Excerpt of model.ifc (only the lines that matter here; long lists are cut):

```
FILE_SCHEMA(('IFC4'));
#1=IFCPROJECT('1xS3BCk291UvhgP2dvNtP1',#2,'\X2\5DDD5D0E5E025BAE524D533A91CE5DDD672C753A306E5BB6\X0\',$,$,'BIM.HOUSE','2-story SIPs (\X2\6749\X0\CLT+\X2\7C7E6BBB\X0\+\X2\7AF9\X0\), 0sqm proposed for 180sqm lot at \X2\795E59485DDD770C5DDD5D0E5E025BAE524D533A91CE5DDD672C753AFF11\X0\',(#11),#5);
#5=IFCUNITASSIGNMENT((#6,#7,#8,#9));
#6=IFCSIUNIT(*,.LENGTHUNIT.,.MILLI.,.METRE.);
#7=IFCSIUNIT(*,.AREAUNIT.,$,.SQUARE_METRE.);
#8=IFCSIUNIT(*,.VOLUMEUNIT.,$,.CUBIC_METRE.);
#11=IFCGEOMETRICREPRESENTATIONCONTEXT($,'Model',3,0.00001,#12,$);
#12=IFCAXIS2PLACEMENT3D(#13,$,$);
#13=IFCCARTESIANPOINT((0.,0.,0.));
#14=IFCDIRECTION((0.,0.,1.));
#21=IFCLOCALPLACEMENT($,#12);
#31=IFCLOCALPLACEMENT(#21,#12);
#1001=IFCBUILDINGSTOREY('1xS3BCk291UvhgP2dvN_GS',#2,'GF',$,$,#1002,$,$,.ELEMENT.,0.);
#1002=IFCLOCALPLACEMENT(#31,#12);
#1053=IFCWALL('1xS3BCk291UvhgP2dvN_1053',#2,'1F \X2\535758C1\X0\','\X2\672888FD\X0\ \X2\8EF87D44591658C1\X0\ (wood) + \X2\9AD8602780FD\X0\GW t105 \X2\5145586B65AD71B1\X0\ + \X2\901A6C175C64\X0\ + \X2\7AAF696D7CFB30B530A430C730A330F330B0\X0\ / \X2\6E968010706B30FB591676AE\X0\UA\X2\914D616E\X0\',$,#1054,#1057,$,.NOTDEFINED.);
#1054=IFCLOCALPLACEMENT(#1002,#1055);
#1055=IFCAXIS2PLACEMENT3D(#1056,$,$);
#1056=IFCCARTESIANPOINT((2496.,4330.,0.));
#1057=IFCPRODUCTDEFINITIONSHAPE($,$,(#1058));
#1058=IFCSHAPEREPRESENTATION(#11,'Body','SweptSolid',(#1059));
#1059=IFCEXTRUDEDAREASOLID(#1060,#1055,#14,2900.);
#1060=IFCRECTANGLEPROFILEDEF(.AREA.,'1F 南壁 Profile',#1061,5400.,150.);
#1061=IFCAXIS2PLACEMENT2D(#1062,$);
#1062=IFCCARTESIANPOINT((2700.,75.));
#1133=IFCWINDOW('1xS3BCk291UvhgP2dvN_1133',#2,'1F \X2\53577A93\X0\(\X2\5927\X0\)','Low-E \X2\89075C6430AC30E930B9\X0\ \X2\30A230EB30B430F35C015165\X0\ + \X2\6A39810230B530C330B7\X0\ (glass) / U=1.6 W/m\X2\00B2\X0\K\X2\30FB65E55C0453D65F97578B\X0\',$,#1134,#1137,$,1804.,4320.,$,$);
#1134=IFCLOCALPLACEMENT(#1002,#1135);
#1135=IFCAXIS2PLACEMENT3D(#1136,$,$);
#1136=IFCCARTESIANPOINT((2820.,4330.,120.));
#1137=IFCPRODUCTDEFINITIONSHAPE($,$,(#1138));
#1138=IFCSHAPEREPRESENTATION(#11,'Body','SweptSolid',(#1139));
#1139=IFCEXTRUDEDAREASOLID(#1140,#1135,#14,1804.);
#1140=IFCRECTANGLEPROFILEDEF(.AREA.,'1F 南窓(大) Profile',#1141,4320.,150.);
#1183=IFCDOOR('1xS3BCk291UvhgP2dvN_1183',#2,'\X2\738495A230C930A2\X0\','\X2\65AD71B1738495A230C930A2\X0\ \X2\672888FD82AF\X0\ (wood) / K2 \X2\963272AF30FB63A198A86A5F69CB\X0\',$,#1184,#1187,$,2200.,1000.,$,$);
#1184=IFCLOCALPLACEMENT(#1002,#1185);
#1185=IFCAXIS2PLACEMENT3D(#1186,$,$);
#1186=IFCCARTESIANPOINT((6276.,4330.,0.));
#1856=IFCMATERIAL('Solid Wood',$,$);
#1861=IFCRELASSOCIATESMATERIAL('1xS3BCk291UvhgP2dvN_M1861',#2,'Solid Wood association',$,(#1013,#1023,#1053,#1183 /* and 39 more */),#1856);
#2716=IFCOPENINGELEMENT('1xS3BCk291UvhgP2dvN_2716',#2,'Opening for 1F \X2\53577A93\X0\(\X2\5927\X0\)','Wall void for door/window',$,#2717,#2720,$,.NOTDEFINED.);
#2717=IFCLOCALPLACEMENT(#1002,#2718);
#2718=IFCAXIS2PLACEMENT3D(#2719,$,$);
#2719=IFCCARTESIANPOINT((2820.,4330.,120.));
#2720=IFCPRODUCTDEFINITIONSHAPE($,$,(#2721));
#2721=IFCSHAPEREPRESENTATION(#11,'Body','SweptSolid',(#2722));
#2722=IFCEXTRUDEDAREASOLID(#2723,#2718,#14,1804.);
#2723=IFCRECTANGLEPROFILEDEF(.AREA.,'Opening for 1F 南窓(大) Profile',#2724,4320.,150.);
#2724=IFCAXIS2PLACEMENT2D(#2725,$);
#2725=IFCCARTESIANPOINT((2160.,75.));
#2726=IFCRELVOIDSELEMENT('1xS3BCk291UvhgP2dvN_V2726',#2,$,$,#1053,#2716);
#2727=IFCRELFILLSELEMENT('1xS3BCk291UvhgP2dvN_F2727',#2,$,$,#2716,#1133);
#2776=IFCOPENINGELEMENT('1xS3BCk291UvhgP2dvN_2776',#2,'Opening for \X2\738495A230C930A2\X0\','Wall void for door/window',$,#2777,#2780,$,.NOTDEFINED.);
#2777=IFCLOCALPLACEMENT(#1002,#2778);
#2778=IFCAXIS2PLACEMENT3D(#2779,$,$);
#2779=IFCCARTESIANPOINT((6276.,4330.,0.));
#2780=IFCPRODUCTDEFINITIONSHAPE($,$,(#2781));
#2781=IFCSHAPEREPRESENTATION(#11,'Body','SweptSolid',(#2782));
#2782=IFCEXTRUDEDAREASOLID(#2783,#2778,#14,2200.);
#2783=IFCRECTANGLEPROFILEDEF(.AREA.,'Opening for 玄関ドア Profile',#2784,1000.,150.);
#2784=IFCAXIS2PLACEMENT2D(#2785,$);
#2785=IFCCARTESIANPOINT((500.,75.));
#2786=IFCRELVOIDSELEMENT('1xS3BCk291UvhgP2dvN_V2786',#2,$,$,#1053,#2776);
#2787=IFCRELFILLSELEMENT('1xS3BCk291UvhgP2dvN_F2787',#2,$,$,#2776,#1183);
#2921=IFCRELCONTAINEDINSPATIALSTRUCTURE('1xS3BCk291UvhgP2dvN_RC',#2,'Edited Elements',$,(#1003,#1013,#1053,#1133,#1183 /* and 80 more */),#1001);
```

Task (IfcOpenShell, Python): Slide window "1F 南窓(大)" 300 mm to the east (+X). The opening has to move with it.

```python
import ifcopenshell
import ifcopenshell.api.geometry
import ifcopenshell.util.placement

model = ifcopenshell.open("model.ifc")

window = model.by_guid("1xS3BCk291UvhgP2dvN_1133")
opening = window.FillsVoids[0].RelatingOpeningElement
wall = opening.VoidsElements[0].RelatingBuildingElement

wall_matrix = ifcopenshell.util.placement.get_local_placement(wall.ObjectPlacement)
shift = wall_matrix[:3, 0] * 300.0
before = ifcopenshell.util.placement.get_local_placement(window.ObjectPlacement)[:3, 3].copy()

# The window is not placed relative to its opening, so move both.
for product in (opening, window):
    matrix = ifcopenshell.util.placement.get_local_placement(product.ObjectPlacement)
    matrix[:3, 3] += shift
    ifcopenshell.api.geometry.edit_object_placement(model, product=product, matrix=matrix, is_si=False)

after = ifcopenshell.util.placement.get_local_placement(window.ObjectPlacement)[:3, 3]
print("window moved by", (after - before).round(3) + 0.0)

model.write("model-out.ifc")
```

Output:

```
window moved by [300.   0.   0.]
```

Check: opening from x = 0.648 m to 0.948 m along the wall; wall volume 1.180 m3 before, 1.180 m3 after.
